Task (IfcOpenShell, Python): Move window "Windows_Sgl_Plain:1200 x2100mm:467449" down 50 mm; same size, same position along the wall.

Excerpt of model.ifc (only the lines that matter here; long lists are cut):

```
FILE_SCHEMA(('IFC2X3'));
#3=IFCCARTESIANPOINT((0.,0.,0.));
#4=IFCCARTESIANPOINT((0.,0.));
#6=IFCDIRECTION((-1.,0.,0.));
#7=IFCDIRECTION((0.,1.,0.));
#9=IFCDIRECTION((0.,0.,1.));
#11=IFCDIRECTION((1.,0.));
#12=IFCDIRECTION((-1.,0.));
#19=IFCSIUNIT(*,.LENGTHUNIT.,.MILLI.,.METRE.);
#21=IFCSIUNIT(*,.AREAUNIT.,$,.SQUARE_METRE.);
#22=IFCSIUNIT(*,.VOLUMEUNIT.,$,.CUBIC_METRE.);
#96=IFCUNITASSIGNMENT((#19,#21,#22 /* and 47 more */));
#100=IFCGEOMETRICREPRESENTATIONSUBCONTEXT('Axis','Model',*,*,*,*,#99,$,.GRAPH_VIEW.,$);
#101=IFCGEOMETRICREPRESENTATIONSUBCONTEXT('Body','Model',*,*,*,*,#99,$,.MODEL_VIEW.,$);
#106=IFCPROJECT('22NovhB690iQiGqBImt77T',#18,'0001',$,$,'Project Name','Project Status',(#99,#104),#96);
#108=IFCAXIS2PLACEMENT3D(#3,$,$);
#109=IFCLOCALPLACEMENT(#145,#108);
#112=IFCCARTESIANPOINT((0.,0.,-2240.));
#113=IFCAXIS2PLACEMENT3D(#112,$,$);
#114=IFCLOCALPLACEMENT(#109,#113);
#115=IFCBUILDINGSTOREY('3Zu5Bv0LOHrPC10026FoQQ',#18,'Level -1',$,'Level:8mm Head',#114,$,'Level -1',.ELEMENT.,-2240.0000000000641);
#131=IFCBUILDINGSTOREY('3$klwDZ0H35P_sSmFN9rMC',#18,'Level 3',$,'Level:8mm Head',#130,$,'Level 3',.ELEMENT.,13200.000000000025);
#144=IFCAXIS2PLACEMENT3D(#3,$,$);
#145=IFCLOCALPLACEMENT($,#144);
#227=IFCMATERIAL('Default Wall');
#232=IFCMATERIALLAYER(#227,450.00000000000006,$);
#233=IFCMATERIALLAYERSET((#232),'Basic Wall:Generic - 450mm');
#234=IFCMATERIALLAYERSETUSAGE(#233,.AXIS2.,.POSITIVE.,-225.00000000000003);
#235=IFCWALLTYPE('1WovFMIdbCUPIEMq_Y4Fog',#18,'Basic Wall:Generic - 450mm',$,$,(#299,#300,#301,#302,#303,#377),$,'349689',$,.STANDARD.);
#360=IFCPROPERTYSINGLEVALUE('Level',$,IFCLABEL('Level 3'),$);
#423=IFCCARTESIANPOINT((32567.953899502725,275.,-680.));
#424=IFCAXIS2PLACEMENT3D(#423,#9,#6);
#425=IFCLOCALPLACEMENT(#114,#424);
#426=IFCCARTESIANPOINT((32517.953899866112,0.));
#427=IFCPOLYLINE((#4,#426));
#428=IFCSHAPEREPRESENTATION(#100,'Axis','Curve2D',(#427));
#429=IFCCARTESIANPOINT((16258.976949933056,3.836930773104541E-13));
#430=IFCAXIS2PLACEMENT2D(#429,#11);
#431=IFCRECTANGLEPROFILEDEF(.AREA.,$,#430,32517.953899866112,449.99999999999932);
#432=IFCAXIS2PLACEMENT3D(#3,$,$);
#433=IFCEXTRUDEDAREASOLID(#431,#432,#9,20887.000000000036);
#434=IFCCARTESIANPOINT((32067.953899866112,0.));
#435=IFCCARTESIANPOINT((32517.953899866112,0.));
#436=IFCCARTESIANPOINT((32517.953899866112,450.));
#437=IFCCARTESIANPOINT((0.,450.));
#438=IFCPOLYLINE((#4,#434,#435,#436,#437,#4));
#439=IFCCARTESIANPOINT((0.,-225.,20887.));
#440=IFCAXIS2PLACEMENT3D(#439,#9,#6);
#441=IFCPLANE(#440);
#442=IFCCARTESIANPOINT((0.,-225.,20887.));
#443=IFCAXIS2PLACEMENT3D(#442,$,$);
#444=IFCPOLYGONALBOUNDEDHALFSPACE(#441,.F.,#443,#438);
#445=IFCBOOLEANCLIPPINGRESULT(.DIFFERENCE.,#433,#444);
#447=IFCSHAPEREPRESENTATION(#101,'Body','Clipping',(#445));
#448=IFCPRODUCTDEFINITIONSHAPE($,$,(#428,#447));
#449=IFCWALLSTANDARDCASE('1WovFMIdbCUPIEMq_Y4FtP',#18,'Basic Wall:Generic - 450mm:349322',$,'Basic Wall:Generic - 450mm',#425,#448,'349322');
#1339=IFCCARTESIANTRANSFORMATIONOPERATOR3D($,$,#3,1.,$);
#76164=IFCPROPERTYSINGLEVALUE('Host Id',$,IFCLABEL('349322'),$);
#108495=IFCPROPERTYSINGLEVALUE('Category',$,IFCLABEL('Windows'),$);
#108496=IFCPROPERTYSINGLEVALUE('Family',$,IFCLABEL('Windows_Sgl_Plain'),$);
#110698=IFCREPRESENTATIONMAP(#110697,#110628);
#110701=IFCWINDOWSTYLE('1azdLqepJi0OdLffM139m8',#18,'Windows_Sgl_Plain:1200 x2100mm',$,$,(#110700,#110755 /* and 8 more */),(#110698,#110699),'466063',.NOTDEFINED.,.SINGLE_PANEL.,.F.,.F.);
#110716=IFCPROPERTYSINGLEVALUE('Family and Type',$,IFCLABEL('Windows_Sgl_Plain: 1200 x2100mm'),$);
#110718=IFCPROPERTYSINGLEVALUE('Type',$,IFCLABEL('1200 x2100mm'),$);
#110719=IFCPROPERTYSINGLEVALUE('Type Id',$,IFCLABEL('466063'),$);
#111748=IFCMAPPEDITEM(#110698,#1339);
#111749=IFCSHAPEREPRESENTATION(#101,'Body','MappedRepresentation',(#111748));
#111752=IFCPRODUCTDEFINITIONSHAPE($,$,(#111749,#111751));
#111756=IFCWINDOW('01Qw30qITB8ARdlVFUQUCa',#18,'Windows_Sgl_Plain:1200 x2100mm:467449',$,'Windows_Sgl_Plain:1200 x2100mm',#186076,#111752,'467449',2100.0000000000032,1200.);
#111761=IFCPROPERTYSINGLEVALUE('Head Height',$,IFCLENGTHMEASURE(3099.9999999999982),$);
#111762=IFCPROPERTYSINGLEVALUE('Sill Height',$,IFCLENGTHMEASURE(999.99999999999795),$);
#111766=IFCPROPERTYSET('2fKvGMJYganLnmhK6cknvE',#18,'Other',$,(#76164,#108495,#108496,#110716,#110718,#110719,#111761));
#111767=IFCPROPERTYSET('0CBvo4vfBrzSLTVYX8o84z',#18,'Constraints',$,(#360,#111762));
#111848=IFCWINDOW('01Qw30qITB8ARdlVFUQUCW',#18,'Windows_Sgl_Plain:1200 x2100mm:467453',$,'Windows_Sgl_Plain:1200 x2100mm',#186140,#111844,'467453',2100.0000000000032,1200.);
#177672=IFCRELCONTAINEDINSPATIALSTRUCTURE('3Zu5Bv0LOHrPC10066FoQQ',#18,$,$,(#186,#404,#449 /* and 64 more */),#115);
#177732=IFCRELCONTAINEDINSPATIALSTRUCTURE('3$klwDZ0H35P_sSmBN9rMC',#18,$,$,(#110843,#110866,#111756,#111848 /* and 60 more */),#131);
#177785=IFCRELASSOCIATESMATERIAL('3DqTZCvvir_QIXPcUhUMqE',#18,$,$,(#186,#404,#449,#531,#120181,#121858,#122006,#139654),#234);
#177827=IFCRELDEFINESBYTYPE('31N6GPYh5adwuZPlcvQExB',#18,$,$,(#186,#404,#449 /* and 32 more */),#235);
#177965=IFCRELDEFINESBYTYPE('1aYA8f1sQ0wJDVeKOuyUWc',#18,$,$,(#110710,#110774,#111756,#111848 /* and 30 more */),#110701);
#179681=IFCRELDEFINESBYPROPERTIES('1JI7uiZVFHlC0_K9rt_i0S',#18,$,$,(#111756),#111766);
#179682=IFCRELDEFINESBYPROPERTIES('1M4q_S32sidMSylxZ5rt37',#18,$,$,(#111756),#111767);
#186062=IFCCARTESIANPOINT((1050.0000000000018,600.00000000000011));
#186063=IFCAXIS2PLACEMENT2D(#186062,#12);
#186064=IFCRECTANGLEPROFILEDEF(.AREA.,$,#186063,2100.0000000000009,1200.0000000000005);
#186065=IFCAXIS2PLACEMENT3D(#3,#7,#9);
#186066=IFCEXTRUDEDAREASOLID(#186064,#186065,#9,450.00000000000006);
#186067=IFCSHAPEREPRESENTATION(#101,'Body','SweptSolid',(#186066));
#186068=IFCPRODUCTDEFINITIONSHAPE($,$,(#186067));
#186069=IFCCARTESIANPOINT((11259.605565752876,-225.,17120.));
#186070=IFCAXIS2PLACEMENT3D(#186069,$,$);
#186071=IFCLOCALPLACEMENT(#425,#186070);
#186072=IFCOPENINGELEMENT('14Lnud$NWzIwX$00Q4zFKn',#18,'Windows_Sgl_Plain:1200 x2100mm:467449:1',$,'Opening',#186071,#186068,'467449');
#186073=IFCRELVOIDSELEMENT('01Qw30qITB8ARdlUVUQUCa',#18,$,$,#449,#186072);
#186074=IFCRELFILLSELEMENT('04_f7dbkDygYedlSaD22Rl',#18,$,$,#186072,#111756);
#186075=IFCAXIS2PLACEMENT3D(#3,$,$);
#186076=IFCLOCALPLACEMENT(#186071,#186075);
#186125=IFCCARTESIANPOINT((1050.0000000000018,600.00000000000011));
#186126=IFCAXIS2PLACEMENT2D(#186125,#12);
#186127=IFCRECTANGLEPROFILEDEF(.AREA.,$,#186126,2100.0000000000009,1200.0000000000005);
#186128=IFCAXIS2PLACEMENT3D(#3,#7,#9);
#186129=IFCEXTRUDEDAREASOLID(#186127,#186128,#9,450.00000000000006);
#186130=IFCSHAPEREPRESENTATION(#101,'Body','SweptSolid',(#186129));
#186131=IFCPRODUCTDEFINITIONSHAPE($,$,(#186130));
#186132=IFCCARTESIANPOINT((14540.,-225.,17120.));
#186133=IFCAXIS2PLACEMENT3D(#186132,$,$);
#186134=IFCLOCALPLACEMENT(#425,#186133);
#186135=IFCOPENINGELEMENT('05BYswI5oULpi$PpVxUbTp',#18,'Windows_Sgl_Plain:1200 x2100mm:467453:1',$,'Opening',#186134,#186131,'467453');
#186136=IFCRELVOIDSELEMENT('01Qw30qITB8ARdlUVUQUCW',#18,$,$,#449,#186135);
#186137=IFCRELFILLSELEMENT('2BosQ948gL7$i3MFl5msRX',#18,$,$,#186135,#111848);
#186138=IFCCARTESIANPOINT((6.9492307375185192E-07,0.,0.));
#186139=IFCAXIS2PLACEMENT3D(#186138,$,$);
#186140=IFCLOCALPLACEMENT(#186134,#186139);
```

```python
import numpy as np
import ifcopenshell
import ifcopenshell.api.geometry
import ifcopenshell.api.pset
import ifcopenshell.util.element
import ifcopenshell.util.placement
import ifcopenshell.util.unit

model = ifcopenshell.open("model.ifc")
unit_scale = ifcopenshell.util.unit.calculate_unit_scale(model)

window = model.by_guid("01Qw30qITB8ARdlVFUQUCa")
opening = window.FillsVoids[0].RelatingOpeningElement
dz = -50.0

shift = np.array([0.0, 0.0, dz])
# The window is placed relative to its opening, so it follows when the opening moves.
matrix = ifcopenshell.util.placement.get_local_placement(opening.ObjectPlacement)
matrix[:3, 3] += shift
ifcopenshell.api.geometry.edit_object_placement(
    model, product=opening, matrix=matrix, is_si=False, should_transform_children=True
)

# Keep the stored heights in step.
pset = model.by_id(ifcopenshell.util.element.get_pset(window, "Other", should_inherit=False)["id"])
ifcopenshell.api.pset.edit_pset(model, pset=pset, properties={
    "Head Height": model.create_entity("IfcLengthMeasure", ifcopenshell.util.element.get_pset(window, "Other", "Head Height") + dz),
})
pset = model.by_id(ifcopenshell.util.element.get_pset(window, "Constraints", should_inherit=False)["id"])
ifcopenshell.api.pset.edit_pset(model, pset=pset, properties={
    "Sill Height": model.create_entity("IfcLengthMeasure", ifcopenshell.util.element.get_pset(window, "Constraints", "Sill Height") + dz),
})

print(f"moved by {dz * unit_scale:+.3f} m")

model.write("model_edited.ifc")
```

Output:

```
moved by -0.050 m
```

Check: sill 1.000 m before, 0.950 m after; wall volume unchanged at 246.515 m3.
